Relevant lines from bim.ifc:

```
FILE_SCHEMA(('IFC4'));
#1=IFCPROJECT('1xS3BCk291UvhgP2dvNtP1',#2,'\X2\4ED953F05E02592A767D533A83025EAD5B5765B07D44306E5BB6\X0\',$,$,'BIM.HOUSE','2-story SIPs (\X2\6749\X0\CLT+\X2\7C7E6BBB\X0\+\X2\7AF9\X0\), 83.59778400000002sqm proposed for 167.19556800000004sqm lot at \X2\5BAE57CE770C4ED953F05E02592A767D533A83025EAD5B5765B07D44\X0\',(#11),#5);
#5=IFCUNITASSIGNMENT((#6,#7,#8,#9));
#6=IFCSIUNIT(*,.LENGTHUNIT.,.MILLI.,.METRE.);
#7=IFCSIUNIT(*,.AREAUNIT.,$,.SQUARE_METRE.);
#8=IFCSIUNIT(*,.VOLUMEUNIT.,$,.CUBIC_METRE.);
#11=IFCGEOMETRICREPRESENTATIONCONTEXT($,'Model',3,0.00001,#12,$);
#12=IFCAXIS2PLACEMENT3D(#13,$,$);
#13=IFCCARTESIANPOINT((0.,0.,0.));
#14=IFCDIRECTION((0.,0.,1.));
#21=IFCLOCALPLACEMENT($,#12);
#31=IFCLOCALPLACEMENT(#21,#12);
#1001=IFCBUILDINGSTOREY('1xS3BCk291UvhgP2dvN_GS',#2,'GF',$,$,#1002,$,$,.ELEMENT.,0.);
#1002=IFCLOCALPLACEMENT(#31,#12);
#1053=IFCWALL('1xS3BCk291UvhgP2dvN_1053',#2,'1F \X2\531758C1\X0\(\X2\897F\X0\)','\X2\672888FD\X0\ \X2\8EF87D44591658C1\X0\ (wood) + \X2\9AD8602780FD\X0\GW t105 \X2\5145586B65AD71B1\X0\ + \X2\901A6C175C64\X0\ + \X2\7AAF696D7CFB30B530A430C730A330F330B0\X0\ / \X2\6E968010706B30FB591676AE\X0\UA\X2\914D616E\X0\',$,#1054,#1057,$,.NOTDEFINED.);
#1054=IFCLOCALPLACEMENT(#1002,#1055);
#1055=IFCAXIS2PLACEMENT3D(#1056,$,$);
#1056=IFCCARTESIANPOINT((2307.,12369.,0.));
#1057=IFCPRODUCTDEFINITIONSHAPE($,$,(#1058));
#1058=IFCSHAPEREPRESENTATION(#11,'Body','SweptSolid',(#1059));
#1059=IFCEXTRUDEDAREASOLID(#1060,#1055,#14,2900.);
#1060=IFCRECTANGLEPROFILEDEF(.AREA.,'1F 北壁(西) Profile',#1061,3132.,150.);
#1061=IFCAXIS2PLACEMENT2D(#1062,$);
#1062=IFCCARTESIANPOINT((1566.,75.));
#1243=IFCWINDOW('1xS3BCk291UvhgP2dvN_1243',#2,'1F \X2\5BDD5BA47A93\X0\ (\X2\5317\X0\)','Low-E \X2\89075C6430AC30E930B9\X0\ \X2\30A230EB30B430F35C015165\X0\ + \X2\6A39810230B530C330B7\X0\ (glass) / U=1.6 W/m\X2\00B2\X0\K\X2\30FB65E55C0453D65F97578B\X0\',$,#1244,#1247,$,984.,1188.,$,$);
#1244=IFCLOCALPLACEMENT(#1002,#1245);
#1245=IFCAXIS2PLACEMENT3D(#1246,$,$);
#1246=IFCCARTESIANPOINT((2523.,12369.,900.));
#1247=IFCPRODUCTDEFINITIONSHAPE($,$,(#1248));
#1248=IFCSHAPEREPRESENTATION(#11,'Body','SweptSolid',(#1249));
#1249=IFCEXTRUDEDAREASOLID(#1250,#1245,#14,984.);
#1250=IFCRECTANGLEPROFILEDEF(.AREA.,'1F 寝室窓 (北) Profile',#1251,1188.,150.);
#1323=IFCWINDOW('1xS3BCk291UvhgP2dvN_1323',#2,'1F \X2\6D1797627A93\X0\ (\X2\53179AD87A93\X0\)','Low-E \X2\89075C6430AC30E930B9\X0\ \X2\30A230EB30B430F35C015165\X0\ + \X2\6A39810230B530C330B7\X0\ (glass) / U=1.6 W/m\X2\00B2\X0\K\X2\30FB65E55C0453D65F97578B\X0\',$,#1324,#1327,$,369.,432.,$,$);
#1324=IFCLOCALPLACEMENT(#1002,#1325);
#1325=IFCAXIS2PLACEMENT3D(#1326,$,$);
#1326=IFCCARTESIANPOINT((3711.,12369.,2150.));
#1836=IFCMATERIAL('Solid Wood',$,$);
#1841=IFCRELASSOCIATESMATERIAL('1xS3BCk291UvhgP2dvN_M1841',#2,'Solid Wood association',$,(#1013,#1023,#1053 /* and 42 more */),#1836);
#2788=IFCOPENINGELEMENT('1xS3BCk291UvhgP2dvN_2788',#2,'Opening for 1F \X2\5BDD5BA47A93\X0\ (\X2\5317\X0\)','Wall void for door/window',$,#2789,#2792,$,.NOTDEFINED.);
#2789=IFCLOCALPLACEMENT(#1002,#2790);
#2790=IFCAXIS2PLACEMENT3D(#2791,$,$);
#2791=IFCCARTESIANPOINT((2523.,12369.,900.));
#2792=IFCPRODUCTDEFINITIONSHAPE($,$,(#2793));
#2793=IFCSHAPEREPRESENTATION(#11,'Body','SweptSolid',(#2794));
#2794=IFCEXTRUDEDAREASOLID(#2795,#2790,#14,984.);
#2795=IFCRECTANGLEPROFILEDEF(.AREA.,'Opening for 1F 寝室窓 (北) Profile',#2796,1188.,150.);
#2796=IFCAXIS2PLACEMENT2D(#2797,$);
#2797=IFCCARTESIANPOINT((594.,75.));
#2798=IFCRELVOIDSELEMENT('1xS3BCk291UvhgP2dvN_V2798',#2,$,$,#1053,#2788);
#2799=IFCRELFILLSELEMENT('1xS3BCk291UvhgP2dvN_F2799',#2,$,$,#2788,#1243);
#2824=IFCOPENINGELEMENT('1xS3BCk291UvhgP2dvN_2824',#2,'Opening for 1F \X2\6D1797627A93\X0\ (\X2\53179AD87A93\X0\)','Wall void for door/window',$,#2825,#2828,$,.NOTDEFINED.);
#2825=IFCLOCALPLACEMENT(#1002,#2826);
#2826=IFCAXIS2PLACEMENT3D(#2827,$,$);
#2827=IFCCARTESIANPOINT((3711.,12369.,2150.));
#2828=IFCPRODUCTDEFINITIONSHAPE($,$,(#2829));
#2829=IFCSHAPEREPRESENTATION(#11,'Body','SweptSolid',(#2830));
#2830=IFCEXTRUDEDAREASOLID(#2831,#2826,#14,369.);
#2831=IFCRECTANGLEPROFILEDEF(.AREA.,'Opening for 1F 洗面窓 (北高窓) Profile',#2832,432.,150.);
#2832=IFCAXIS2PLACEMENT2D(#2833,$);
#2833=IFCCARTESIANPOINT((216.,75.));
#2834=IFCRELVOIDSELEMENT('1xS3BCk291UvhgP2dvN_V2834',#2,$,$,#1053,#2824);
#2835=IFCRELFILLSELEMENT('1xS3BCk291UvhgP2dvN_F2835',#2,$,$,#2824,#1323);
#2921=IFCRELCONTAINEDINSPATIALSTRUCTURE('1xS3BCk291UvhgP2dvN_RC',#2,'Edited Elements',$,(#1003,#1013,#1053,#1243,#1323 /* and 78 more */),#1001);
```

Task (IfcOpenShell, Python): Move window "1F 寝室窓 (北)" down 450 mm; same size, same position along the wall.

```python
import numpy as np
import ifcopenshell
import ifcopenshell.api.geometry
import ifcopenshell.util.placement
import ifcopenshell.util.unit

model = ifcopenshell.open("bim.ifc")
unit_scale = ifcopenshell.util.unit.calculate_unit_scale(model)

window = model.by_id(1243)
opening = window.FillsVoids[0].RelatingOpeningElement
dz = -450.0

shift = np.array([0.0, 0.0, dz])
# The window is not placed relative to its opening, so move both.
for product in (opening, window):
    matrix = ifcopenshell.util.placement.get_local_placement(product.ObjectPlacement)
    matrix[:3, 3] += shift
    ifcopenshell.api.geometry.edit_object_placement(model, product=product, matrix=matrix, is_si=False)

print(f"moved by {dz * unit_scale:+.3f} m")

model.write("bim_updated.ifc")
```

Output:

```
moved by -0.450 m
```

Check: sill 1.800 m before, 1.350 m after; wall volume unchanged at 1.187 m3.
